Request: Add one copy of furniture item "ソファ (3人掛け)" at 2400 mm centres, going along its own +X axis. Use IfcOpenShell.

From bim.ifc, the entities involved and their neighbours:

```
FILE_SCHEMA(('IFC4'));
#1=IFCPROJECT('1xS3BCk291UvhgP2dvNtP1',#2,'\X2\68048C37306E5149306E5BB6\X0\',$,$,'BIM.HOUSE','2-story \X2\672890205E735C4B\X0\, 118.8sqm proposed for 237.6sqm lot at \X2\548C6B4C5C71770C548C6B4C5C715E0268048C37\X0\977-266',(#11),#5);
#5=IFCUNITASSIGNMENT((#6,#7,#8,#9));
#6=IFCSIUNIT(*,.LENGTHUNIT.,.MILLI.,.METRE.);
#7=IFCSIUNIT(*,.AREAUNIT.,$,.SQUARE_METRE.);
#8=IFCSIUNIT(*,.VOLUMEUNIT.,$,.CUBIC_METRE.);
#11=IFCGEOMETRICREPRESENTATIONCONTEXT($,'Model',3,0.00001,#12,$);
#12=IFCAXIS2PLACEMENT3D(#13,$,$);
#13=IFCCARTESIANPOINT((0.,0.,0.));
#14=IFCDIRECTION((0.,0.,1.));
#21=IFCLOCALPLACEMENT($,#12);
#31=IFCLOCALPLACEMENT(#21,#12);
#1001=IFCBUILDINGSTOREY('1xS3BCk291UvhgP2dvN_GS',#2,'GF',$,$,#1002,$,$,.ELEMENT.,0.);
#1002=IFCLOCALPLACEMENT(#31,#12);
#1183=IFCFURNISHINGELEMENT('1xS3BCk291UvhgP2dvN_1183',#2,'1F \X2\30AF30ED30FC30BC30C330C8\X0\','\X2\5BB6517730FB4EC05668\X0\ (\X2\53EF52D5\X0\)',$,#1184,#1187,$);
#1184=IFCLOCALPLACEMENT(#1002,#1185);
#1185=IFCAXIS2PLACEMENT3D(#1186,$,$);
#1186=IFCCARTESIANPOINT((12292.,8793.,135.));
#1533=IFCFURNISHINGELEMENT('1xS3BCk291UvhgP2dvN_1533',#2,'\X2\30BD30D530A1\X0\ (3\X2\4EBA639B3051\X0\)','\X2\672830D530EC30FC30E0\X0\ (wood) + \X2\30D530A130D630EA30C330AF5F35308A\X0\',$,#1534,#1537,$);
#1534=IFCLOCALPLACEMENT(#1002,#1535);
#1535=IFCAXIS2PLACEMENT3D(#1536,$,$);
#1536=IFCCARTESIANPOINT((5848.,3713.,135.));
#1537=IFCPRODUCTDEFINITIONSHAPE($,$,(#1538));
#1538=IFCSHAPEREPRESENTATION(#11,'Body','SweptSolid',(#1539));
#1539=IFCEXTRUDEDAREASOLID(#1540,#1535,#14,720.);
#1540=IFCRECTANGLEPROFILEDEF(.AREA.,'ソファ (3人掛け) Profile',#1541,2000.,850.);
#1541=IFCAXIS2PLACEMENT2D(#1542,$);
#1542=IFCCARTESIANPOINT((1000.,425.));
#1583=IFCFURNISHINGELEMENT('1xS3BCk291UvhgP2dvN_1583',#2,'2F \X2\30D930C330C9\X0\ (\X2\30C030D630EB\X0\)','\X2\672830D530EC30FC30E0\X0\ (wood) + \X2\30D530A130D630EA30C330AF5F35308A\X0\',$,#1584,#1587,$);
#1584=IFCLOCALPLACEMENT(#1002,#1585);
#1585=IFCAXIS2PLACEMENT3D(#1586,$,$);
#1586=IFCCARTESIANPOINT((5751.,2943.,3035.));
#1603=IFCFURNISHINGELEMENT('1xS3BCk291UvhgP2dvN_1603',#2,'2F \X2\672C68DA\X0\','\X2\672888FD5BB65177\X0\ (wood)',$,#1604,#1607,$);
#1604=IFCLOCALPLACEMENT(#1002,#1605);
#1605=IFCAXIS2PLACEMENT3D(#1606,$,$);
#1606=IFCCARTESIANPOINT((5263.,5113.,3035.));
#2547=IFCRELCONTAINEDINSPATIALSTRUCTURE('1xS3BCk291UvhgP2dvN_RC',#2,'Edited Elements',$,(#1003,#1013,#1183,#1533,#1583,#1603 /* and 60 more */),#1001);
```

```python
import ifcopenshell
import ifcopenshell.api.geometry
import ifcopenshell.api.root
import ifcopenshell.util.element
import ifcopenshell.util.placement
import ifcopenshell.util.unit

model = ifcopenshell.open("bim.ifc")
unit_scale = ifcopenshell.util.unit.calculate_unit_scale(model)


def reuse_history(source, copy):
    """copy_class also copies each property set's owner history, people and application; keep the originals."""
    for rel in copy.IsDefinedBy:
        if rel.is_a("IfcRelDefinesByProperties") and (history := rel.RelatingPropertyDefinition.OwnerHistory):
            rel.RelatingPropertyDefinition.OwnerHistory = source.OwnerHistory
            ifcopenshell.util.element.remove_deep2(model, history)


source = model.by_id(1533)
base = ifcopenshell.util.placement.get_local_placement(source.ObjectPlacement)
step = base[:3, 0] * 2.4 / unit_scale

for i in range(1, 2):
    copy = ifcopenshell.api.root.copy_class(model, product=source)
    copy.Representation = ifcopenshell.util.element.copy_deep(
        model, source.Representation, exclude=["IfcGeometricRepresentationContext", "IfcRepresentationMap"]
    )
    reuse_history(source, copy)
    matrix = base.copy()
    matrix[:3, 3] += i * step
    print("added at", matrix[:3, 3].round(3) + 0.0)
    ifcopenshell.api.geometry.edit_object_placement(model, product=copy, matrix=matrix, is_si=False)

model.write("bim-out.ifc")
```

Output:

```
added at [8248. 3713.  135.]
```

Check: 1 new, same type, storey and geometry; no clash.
